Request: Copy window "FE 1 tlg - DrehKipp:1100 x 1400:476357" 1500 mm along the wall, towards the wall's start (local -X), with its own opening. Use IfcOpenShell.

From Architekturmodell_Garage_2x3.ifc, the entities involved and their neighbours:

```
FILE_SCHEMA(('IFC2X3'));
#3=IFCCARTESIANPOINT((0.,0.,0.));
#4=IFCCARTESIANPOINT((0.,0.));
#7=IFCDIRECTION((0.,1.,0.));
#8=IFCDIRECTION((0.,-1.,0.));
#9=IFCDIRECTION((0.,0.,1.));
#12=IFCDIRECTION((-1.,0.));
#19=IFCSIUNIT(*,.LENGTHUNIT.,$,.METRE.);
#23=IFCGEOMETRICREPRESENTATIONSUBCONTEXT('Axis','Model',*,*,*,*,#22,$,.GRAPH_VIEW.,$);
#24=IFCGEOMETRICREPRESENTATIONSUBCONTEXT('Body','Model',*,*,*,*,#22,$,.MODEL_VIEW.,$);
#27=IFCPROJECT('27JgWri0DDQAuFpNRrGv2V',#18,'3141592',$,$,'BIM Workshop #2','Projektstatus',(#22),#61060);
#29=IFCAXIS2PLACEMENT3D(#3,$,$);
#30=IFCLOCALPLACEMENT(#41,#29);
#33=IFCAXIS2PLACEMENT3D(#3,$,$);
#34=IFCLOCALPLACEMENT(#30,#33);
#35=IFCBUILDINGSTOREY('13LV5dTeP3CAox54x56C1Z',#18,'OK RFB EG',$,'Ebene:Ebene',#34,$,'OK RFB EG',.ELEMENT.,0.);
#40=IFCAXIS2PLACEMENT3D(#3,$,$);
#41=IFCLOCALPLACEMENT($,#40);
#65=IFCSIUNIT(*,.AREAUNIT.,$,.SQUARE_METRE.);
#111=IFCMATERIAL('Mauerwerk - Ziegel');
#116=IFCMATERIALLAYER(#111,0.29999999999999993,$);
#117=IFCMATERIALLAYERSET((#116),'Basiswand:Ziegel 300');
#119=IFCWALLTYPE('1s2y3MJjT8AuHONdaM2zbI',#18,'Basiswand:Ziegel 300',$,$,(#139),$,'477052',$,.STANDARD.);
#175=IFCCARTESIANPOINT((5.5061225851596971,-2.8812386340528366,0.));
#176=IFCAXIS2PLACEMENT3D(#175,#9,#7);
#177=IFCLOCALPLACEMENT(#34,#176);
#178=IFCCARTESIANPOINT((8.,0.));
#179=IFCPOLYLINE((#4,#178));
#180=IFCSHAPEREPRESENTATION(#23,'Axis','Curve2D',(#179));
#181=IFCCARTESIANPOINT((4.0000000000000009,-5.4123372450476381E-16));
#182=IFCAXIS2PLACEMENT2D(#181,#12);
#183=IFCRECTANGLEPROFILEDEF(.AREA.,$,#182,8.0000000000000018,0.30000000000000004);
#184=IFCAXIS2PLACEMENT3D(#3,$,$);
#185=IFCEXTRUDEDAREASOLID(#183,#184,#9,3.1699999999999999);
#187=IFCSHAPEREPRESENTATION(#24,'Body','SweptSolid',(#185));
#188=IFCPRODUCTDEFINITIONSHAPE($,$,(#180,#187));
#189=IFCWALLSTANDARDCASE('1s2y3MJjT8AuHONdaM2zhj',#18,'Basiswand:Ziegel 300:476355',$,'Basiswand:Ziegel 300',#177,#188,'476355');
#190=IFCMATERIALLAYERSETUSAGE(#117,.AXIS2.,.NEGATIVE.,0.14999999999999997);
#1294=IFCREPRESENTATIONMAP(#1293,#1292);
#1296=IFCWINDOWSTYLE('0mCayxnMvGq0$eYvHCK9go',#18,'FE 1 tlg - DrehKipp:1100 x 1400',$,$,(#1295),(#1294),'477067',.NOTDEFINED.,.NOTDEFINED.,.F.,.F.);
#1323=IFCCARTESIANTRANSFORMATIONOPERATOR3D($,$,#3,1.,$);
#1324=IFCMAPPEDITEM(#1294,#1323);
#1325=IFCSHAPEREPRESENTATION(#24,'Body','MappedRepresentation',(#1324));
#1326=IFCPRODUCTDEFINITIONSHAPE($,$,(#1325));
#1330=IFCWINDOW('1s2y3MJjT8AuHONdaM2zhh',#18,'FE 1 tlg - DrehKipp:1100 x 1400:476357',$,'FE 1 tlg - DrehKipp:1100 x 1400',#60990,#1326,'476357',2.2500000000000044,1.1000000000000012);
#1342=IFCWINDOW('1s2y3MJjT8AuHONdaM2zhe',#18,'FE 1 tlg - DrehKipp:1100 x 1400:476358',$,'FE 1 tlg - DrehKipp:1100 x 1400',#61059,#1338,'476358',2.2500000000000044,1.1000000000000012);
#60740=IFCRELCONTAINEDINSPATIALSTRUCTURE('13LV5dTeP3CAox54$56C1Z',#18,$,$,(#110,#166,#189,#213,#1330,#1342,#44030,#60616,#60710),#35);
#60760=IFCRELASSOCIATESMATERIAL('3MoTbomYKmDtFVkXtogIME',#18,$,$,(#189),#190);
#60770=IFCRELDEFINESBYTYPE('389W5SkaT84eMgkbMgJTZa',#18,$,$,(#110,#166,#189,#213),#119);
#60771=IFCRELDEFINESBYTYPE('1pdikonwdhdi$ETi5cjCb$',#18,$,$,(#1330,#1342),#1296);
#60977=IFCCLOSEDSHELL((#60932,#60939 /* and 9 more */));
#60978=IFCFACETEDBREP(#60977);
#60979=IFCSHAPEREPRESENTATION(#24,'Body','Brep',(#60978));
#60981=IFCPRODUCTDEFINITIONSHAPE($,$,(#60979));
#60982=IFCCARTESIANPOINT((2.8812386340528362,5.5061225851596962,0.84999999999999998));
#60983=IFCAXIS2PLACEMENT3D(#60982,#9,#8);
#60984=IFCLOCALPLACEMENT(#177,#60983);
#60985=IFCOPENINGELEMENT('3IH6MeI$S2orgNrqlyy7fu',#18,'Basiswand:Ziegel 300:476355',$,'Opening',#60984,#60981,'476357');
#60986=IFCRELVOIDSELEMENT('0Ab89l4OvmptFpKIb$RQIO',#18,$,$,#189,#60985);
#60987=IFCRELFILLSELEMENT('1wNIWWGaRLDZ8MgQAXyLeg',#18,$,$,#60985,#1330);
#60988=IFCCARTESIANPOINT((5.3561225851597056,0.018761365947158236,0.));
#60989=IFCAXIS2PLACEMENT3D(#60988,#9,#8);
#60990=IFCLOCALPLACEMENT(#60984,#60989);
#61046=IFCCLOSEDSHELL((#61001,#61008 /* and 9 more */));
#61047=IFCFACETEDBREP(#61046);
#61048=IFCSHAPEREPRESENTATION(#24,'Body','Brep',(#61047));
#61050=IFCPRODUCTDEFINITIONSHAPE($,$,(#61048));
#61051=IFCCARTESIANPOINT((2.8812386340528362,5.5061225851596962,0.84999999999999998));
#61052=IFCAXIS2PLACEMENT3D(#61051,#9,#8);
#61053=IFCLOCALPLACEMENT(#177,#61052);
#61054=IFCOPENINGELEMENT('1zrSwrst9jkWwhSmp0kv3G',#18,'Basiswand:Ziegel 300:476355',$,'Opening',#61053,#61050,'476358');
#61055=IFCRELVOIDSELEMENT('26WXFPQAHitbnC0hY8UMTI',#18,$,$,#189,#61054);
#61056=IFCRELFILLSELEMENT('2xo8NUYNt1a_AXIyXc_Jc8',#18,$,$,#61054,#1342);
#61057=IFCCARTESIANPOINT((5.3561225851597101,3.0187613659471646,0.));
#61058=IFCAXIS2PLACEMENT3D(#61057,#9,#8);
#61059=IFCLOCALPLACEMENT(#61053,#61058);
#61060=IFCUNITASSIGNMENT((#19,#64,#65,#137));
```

```python
import ifcopenshell
import ifcopenshell.api.feature
import ifcopenshell.api.geometry
import ifcopenshell.api.root
import ifcopenshell.geom
import ifcopenshell.util.element
import ifcopenshell.util.placement
import ifcopenshell.util.shape

model = ifcopenshell.open("Architekturmodell_Garage_2x3.ifc")
settings = ifcopenshell.geom.settings()


def volume(element):
    """Net volume in cubic metres, openings subtracted."""
    shape = ifcopenshell.geom.create_shape(settings, element)
    return ifcopenshell.util.shape.get_volume(shape.geometry)


def reuse_history(source, copy):
    """copy_class also copies each property set's owner history, people and application; keep the originals."""
    for rel in copy.IsDefinedBy:
        if rel.is_a("IfcRelDefinesByProperties") and (history := rel.RelatingPropertyDefinition.OwnerHistory):
            rel.RelatingPropertyDefinition.OwnerHistory = source.OwnerHistory
            ifcopenshell.util.element.remove_deep2(model, history)


window = model.by_guid("1s2y3MJjT8AuHONdaM2zhh")
opening = window.FillsVoids[0].RelatingOpeningElement
wall = opening.VoidsElements[0].RelatingBuildingElement
before = volume(wall)
shift = ifcopenshell.util.placement.get_local_placement(wall.ObjectPlacement)[:3, 0] * -1.5

# copy_class copies the void relationship, type, container and properties, but no geometry.
new_opening = ifcopenshell.api.root.copy_class(model, product=opening)
new_opening.Representation = ifcopenshell.util.element.copy_deep(
    model, opening.Representation, exclude=["IfcGeometricRepresentationContext", "IfcRepresentationMap"]
)
new_opening.Name = "Basiswand:Ziegel 300"
new_opening.Tag = None
new_window = ifcopenshell.api.root.copy_class(model, product=window)
new_window.Representation = ifcopenshell.util.element.copy_deep(
    model, window.Representation, exclude=["IfcGeometricRepresentationContext", "IfcRepresentationMap"]
)
new_window.Name = "FE 1 tlg - DrehKipp:1100 x 1400"
new_window.Tag = None
reuse_history(window, new_window)
fills = ifcopenshell.api.feature.add_filling(model, opening=new_opening, element=new_window)
fills.OwnerHistory = new_window.OwnerHistory  # required in IFC2X3

for old, new in ((opening, new_opening), (window, new_window)):
    matrix = ifcopenshell.util.placement.get_local_placement(old.ObjectPlacement)
    matrix[:3, 3] += shift
    ifcopenshell.api.geometry.edit_object_placement(model, product=new, matrix=matrix, is_si=False)

after = volume(wall)

print(f"wall volume {before:.3f} -> {after:.3f} m3")

model.write("Architekturmodell_Garage_2x3_updated.ifc")
```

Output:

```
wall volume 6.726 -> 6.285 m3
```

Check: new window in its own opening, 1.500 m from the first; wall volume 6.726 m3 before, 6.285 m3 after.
